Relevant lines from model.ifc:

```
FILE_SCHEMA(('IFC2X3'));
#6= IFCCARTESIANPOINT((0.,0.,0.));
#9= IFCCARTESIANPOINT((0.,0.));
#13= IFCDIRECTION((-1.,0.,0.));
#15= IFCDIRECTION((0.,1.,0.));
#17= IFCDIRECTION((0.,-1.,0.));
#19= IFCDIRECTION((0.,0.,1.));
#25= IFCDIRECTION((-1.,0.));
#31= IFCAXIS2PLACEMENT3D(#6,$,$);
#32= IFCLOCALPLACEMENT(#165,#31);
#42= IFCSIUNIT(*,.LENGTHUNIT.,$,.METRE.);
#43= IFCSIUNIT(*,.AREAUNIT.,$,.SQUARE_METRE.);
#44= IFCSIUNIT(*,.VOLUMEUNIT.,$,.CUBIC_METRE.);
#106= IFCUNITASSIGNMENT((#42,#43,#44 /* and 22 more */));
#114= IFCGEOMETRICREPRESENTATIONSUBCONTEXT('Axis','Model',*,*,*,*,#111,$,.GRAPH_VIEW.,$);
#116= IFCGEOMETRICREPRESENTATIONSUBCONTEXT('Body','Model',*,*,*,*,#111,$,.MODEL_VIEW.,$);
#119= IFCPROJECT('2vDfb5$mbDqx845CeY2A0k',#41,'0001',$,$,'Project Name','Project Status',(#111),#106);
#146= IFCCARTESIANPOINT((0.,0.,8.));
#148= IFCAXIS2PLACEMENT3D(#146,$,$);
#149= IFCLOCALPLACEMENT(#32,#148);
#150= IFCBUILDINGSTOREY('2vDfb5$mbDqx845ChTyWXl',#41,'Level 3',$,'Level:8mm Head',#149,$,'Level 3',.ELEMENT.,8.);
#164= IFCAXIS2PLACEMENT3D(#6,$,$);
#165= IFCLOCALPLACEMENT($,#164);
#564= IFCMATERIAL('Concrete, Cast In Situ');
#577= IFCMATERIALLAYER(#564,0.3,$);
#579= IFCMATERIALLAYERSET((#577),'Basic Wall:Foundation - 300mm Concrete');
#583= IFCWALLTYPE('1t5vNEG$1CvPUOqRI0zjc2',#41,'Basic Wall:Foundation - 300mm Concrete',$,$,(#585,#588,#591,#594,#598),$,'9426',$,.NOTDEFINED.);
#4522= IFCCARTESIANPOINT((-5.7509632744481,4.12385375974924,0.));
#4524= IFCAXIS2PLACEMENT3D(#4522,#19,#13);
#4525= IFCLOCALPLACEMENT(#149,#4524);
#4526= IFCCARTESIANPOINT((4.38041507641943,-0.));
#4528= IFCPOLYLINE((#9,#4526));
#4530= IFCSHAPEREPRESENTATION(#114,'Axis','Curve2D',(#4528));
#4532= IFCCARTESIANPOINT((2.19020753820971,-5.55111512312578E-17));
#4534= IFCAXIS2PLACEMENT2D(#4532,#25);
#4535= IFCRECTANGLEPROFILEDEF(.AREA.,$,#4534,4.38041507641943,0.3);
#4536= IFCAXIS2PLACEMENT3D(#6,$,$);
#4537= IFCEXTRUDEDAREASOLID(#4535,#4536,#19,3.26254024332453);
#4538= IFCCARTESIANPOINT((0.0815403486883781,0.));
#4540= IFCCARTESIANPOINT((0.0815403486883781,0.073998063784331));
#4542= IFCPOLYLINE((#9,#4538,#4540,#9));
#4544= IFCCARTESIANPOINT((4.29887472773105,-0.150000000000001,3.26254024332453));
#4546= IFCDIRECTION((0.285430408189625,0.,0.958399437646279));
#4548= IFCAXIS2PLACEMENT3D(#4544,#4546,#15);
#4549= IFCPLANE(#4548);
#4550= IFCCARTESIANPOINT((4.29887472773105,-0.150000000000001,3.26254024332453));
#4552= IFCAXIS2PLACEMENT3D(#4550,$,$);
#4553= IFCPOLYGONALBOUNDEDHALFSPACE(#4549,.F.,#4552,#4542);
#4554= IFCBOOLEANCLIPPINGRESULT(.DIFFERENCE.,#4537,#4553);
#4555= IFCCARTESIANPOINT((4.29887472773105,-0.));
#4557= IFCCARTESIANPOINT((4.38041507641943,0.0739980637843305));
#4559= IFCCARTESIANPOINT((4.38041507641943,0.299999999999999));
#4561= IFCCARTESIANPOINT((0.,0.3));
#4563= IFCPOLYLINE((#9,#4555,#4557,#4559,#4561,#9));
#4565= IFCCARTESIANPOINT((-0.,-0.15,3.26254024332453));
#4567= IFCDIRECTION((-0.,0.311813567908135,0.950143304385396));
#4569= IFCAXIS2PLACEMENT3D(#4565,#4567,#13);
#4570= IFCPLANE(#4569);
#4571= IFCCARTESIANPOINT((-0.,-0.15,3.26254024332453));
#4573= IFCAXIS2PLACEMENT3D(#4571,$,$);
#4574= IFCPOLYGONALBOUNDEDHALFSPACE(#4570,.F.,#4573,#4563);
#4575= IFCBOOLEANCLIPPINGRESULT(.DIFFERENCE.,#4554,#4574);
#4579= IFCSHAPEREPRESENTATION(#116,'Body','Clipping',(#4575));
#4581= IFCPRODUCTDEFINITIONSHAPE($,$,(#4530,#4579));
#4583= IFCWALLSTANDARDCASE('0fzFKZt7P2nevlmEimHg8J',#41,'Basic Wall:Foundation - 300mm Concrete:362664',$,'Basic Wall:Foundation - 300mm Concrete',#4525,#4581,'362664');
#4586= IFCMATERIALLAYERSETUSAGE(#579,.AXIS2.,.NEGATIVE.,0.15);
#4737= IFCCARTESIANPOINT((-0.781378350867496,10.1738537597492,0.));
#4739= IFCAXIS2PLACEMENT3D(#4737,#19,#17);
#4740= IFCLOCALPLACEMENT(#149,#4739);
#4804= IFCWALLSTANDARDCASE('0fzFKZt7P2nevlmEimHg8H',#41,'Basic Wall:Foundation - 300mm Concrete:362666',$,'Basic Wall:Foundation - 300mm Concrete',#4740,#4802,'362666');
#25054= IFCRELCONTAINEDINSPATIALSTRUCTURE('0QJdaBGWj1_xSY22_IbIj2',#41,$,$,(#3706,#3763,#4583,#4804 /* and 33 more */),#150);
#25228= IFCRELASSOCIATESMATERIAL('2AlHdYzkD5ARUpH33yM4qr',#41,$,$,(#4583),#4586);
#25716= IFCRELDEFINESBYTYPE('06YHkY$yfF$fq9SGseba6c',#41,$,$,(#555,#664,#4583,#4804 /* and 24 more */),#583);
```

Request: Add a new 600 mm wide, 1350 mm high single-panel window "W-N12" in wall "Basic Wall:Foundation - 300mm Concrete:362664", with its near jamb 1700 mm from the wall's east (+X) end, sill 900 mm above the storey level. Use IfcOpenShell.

```python
import numpy as np
import ifcopenshell
import ifcopenshell.api.feature
import ifcopenshell.api.geometry
import ifcopenshell.api.root
import ifcopenshell.api.spatial
import ifcopenshell.api.type
import ifcopenshell.geom
import ifcopenshell.util.element
import ifcopenshell.util.placement
import ifcopenshell.util.representation
import ifcopenshell.util.shape
import ifcopenshell.util.unit

model = ifcopenshell.open("model.ifc")
unit_scale = ifcopenshell.util.unit.calculate_unit_scale(model)
settings = ifcopenshell.geom.settings()


def volume(element):
    """Net volume in cubic metres, openings subtracted."""
    shape = ifcopenshell.geom.create_shape(settings, element)
    return ifcopenshell.util.shape.get_volume(shape.geometry)


wall = model.by_guid("0fzFKZt7P2nevlmEimHg8J")
storey = ifcopenshell.util.element.get_container(wall, ifc_class="IfcBuildingStorey")
context = ifcopenshell.util.representation.get_context(model, "Model", "Body", "MODEL_VIEW")
before = volume(wall)

width, height, from_end, sill = 0.6, 1.35, 1.7, 0.9  # metres

# The wall runs along its own X axis, and the end named is its -X end.
wall_shape = ifcopenshell.geom.create_shape(settings, wall)
x, y, z = ifcopenshell.util.shape.get_vertices(wall_shape.geometry).T
start = x.min() + from_end
face, thickness = float(y.min()), float(y.max() - y.min())
wall_matrix = ifcopenshell.util.placement.get_local_placement(wall.ObjectPlacement)
level = ifcopenshell.util.placement.get_local_placement(storey.ObjectPlacement)[2, 3]


def in_wall(x, y):
    """Placement at x, y metres in the wall's axes, at sill height."""
    matrix = wall_matrix.copy()
    matrix[:, 3] = wall_matrix @ np.array([x / unit_scale, y / unit_scale, 0.0, 1.0])
    matrix[2, 3] = level + sill / unit_scale
    return matrix


# Opening: a box that overshoots both wall faces by 50 mm.
opening = ifcopenshell.api.root.create_entity(model, ifc_class="IfcOpeningElement")
box = ifcopenshell.api.geometry.add_wall_representation(
    model, context=context, length=width, height=height, thickness=thickness + 0.1
)
ifcopenshell.api.geometry.assign_representation(model, product=opening, representation=box)
ifcopenshell.api.geometry.edit_object_placement(model, product=opening, matrix=in_wall(start, face - 0.05), is_si=False)
ifcopenshell.api.feature.add_feature(model, feature=opening, element=wall)

window = ifcopenshell.api.root.create_entity(model, ifc_class="IfcWindow", name="W-N12")
window.OverallWidth, window.OverallHeight = width / unit_scale, height / unit_scale
body = ifcopenshell.api.geometry.add_window_representation(
    model,
    context=context,
    overall_width=window.OverallWidth,
    overall_height=window.OverallHeight,
    partition_type="SINGLE_PANEL",
)
ifcopenshell.api.geometry.assign_representation(model, product=window, representation=body)
ifcopenshell.api.spatial.assign_container(model, products=[window], relating_structure=storey)
fills = ifcopenshell.api.feature.add_filling(model, opening=opening, element=window)
fills.OwnerHistory = window.OwnerHistory  # required in IFC2X3

# IFC2X3 keeps the operation on the window style.
style = ifcopenshell.api.root.create_entity(model, ifc_class="IfcWindowStyle", name="W-N12")
style.OperationType, style.ConstructionType = "SINGLE_PANEL", "NOTDEFINED"
style.ParameterTakesPrecedence = style.Sizeable = False
ifcopenshell.api.type.assign_type(model, related_objects=[window], relating_type=style)

# Centre the window in the wall's thickness.
ifcopenshell.api.geometry.edit_object_placement(model, product=window, matrix=in_wall(start, face), is_si=False)
window_shape = ifcopenshell.geom.create_shape(settings, window)
depth = ifcopenshell.util.shape.get_vertices(window_shape.geometry)[:, 1]
offset = face + thickness / 2 - (depth.min() + depth.max()) / 2
ifcopenshell.api.geometry.edit_object_placement(model, product=window, matrix=in_wall(start, offset), is_si=False)

after = volume(wall)

print(f"wall volume {before:.3f} -> {after:.3f} m3")

model.write("model-out.ifc")
```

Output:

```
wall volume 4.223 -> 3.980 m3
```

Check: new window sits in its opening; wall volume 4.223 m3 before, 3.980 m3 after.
